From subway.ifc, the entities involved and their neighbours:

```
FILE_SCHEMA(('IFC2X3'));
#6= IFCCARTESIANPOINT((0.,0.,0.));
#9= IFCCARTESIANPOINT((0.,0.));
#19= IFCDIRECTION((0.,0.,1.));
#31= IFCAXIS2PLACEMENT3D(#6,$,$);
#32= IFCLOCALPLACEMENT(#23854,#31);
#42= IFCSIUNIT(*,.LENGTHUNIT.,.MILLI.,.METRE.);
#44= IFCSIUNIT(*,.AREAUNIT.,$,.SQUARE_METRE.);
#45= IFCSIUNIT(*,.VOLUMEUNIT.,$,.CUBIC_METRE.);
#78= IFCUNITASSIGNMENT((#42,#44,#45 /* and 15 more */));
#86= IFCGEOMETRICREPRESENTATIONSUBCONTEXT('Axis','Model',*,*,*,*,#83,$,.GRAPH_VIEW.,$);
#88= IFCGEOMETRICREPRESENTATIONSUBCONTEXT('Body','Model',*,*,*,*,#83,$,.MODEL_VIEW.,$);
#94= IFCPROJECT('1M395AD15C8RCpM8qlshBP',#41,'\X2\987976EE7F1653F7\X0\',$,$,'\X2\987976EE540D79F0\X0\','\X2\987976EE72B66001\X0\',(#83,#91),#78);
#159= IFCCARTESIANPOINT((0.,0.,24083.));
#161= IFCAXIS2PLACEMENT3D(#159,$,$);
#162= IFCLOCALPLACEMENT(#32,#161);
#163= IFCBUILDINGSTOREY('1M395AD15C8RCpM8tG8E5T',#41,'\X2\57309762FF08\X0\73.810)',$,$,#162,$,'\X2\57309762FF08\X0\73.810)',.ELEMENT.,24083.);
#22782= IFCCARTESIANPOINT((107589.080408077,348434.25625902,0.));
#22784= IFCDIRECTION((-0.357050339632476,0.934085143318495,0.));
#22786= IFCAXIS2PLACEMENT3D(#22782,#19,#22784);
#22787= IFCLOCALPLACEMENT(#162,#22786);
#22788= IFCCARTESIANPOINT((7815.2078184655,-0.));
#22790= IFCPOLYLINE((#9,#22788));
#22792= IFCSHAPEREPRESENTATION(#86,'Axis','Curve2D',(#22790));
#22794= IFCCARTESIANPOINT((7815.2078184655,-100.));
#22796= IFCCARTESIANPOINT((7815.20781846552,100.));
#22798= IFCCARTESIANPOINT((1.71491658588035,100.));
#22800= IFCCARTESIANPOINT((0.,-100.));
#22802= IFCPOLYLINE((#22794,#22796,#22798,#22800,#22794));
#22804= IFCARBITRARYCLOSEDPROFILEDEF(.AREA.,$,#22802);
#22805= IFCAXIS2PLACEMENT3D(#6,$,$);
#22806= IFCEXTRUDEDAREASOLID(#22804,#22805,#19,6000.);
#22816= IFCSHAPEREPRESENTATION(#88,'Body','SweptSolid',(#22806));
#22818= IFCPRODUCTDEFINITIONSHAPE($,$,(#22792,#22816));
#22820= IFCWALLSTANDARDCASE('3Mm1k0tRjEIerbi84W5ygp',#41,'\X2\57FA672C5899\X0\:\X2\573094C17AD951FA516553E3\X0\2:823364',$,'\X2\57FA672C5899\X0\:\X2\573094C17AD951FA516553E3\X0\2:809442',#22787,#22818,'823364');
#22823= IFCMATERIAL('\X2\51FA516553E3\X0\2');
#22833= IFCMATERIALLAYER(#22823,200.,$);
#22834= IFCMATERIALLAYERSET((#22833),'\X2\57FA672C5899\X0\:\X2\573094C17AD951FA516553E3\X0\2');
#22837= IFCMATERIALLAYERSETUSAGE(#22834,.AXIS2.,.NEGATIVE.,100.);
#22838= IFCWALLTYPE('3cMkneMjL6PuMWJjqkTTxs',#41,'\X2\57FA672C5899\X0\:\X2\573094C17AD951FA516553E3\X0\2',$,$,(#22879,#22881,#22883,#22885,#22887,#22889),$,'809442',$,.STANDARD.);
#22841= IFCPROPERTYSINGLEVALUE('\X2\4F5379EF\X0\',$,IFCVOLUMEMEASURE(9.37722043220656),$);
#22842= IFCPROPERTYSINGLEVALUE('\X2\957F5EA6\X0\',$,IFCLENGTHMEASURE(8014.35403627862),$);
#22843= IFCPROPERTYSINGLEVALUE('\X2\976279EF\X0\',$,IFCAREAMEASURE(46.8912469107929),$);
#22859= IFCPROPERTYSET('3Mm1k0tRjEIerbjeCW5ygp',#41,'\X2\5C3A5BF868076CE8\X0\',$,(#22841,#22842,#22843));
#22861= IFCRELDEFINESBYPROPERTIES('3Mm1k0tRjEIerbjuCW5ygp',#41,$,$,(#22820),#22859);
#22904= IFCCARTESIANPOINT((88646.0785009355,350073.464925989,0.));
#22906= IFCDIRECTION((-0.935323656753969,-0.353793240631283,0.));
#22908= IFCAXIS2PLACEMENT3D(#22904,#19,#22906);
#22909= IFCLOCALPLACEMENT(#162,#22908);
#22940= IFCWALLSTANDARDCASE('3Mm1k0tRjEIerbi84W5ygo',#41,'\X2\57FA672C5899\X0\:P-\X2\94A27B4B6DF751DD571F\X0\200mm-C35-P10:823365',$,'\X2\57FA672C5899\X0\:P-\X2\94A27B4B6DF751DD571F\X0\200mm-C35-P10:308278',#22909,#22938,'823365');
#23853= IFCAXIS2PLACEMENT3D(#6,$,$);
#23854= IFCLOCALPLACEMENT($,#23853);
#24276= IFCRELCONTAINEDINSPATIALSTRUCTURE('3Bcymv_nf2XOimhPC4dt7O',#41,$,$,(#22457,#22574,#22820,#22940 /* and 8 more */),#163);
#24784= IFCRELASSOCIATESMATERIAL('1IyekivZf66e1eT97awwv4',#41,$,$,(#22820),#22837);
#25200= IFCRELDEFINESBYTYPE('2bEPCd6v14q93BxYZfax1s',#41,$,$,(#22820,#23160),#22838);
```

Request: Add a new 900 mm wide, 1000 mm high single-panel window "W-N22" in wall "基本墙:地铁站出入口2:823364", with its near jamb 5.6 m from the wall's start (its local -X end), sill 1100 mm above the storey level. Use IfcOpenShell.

```python
import numpy as np
import ifcopenshell
import ifcopenshell.api.feature
import ifcopenshell.api.geometry
import ifcopenshell.api.pset
import ifcopenshell.api.root
import ifcopenshell.api.spatial
import ifcopenshell.api.type
import ifcopenshell.geom
import ifcopenshell.util.element
import ifcopenshell.util.placement
import ifcopenshell.util.representation
import ifcopenshell.util.shape
import ifcopenshell.util.unit

model = ifcopenshell.open("subway.ifc")
unit_scale = ifcopenshell.util.unit.calculate_unit_scale(model)
area_scale = ifcopenshell.util.unit.calculate_unit_scale(model, "AREAUNIT")
volume_scale = ifcopenshell.util.unit.calculate_unit_scale(model, "VOLUMEUNIT")
settings = ifcopenshell.geom.settings()


def volume(element):
    """Net volume in cubic metres, openings subtracted."""
    shape = ifcopenshell.geom.create_shape(settings, element)
    return ifcopenshell.util.shape.get_volume(shape.geometry)


wall = model.by_id(22820)
storey = ifcopenshell.util.element.get_container(wall, ifc_class="IfcBuildingStorey")
context = ifcopenshell.util.representation.get_context(model, "Model", "Body", "MODEL_VIEW")
before = volume(wall)

width, height, from_end, sill = 0.9, 1, 5.6, 1.1  # metres

# The wall runs along its own X axis, and the end named is its -X end.
wall_shape = ifcopenshell.geom.create_shape(settings, wall)
x, y, z = ifcopenshell.util.shape.get_vertices(wall_shape.geometry).T
start = x.min() + from_end
face, thickness = float(y.min()), float(y.max() - y.min())
wall_matrix = ifcopenshell.util.placement.get_local_placement(wall.ObjectPlacement)
level = ifcopenshell.util.placement.get_local_placement(storey.ObjectPlacement)[2, 3]


def in_wall(x, y):
    """Placement at x, y metres in the wall's axes, at sill height."""
    matrix = wall_matrix.copy()
    matrix[:, 3] = wall_matrix @ np.array([x / unit_scale, y / unit_scale, 0.0, 1.0])
    matrix[2, 3] = level + sill / unit_scale
    return matrix


# Opening: a box that overshoots both wall faces by 50 mm.
opening = ifcopenshell.api.root.create_entity(model, ifc_class="IfcOpeningElement")
box = ifcopenshell.api.geometry.add_wall_representation(
    model, context=context, length=width, height=height, thickness=thickness + 0.1
)
ifcopenshell.api.geometry.assign_representation(model, product=opening, representation=box)
ifcopenshell.api.geometry.edit_object_placement(model, product=opening, matrix=in_wall(start, face - 0.05), is_si=False)
ifcopenshell.api.feature.add_feature(model, feature=opening, element=wall)

window = ifcopenshell.api.root.create_entity(model, ifc_class="IfcWindow", name="W-N22")
window.OverallWidth, window.OverallHeight = width / unit_scale, height / unit_scale
body = ifcopenshell.api.geometry.add_window_representation(
    model,
    context=context,
    overall_width=window.OverallWidth,
    overall_height=window.OverallHeight,
    partition_type="SINGLE_PANEL",
)
ifcopenshell.api.geometry.assign_representation(model, product=window, representation=body)
ifcopenshell.api.spatial.assign_container(model, products=[window], relating_structure=storey)
fills = ifcopenshell.api.feature.add_filling(model, opening=opening, element=window)
fills.OwnerHistory = window.OwnerHistory  # required in IFC2X3

# IFC2X3 keeps the operation on the window style.
style = ifcopenshell.api.root.create_entity(model, ifc_class="IfcWindowStyle", name="W-N22")
style.OperationType, style.ConstructionType = "SINGLE_PANEL", "NOTDEFINED"
style.ParameterTakesPrecedence = style.Sizeable = False
ifcopenshell.api.type.assign_type(model, related_objects=[window], relating_type=style)

# Centre the window in the wall's thickness.
ifcopenshell.api.geometry.edit_object_placement(model, product=window, matrix=in_wall(start, face), is_si=False)
window_shape = ifcopenshell.geom.create_shape(settings, window)
depth = ifcopenshell.util.shape.get_vertices(window_shape.geometry)[:, 1]
offset = face + thickness / 2 - (depth.min() + depth.max()) / 2
ifcopenshell.api.geometry.edit_object_placement(model, product=window, matrix=in_wall(start, offset), is_si=False)

after = volume(wall)

# Update the wall's stored quantities.
pset = model.by_id(ifcopenshell.util.element.get_pset(wall, "尺寸标注", should_inherit=False)["id"])
ifcopenshell.api.pset.edit_pset(model, pset=pset, properties={
    "体积": model.create_entity("IfcVolumeMeasure", after / volume_scale),
    "面积": model.create_entity("IfcAreaMeasure", after / thickness / area_scale),
})

print(f"wall volume {before:.3f} -> {after:.3f} m3")

model.write("subway_rev.ifc")
```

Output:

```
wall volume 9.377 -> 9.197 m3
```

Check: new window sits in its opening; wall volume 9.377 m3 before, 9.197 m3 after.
